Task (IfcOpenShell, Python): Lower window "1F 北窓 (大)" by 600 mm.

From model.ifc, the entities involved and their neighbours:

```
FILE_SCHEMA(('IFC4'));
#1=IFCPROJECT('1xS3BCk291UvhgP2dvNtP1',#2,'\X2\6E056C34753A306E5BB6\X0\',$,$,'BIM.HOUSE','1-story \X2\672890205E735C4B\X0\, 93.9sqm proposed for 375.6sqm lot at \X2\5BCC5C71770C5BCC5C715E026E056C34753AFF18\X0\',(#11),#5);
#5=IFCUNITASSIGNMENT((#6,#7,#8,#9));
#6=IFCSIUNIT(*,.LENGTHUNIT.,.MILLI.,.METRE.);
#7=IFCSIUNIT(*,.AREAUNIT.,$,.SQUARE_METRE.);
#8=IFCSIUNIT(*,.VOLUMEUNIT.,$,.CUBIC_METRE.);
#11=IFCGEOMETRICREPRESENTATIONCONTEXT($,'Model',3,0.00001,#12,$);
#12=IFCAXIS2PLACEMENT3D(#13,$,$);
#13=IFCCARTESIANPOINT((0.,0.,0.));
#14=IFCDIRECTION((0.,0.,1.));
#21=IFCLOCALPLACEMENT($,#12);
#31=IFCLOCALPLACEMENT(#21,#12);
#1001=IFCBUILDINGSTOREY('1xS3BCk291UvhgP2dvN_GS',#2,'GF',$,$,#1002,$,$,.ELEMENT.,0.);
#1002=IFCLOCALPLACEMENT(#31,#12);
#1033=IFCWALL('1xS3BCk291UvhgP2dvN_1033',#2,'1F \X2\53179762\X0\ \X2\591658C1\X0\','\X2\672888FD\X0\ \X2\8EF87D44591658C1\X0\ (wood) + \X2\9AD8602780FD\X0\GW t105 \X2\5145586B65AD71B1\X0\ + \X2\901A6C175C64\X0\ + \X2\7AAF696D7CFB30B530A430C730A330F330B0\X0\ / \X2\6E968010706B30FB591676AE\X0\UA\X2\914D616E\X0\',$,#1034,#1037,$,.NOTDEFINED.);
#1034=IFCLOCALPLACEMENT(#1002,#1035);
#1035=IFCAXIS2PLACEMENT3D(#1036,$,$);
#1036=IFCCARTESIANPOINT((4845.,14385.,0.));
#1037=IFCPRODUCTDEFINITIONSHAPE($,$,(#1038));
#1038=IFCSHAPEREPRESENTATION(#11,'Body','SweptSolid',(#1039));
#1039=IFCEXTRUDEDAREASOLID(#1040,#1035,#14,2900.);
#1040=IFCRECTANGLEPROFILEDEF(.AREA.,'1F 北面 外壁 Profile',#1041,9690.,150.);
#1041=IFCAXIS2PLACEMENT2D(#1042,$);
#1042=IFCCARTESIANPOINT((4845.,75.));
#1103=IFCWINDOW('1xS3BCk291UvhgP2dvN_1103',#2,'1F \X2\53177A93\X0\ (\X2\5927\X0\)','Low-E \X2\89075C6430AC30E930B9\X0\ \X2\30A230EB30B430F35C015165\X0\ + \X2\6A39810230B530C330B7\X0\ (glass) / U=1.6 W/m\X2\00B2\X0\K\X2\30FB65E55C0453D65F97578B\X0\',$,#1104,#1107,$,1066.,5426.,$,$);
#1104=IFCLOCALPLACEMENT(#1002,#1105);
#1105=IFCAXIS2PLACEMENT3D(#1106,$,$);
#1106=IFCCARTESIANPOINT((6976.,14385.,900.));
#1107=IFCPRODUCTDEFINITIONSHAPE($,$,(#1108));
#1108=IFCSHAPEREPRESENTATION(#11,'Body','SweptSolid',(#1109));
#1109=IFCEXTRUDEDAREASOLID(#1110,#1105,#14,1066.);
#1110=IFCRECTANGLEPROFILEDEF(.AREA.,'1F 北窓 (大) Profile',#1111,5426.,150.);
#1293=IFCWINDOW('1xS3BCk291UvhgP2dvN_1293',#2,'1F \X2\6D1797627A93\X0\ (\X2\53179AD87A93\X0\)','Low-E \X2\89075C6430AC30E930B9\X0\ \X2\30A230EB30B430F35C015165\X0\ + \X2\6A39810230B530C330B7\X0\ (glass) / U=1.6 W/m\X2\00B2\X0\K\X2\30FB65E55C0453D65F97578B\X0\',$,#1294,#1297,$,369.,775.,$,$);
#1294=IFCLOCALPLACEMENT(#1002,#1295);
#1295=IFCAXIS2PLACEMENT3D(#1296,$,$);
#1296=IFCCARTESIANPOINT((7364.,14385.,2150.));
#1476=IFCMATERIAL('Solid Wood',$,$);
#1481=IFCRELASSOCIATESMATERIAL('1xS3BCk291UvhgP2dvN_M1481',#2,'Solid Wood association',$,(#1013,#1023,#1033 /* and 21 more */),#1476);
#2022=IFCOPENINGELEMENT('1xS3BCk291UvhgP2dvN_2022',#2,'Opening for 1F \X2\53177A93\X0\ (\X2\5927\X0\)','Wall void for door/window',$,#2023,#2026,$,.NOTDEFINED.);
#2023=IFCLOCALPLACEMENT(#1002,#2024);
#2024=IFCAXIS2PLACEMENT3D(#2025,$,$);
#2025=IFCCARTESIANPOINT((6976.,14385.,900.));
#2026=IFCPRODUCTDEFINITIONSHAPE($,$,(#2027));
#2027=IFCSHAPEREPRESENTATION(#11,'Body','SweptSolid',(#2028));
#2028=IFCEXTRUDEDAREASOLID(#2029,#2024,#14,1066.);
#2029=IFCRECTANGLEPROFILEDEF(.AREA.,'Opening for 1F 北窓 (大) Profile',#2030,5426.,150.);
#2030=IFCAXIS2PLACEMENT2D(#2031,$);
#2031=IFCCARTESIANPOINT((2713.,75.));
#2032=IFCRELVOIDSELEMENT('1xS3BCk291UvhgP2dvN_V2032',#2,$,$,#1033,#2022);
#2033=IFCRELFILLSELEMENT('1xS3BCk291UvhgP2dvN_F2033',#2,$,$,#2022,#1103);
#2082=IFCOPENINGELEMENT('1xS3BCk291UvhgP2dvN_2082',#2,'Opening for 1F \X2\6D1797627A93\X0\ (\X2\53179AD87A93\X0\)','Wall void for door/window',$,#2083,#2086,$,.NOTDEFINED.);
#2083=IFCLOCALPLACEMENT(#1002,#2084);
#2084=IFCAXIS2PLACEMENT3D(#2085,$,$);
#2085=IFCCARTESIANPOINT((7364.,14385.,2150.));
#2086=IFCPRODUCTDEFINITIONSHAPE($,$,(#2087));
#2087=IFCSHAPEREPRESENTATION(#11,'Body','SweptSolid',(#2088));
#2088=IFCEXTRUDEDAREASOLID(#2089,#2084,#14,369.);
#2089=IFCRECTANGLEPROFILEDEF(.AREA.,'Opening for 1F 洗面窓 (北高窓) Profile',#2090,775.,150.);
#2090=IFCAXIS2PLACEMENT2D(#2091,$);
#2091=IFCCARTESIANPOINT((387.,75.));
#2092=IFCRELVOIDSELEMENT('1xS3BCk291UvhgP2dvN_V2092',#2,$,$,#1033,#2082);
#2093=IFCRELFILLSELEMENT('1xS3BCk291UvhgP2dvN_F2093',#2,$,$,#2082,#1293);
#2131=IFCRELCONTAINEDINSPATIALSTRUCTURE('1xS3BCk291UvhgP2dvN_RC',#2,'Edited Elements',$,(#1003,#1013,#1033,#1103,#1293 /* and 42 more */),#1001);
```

```python
import numpy as np
import ifcopenshell
import ifcopenshell.api.geometry
import ifcopenshell.util.placement
import ifcopenshell.util.unit

model = ifcopenshell.open("model.ifc")
unit_scale = ifcopenshell.util.unit.calculate_unit_scale(model)

window = model.by_guid("1xS3BCk291UvhgP2dvN_1103")
opening = window.FillsVoids[0].RelatingOpeningElement
dz = -600.0

shift = np.array([0.0, 0.0, dz])
# The window is not placed relative to its opening, so move both.
for product in (opening, window):
    matrix = ifcopenshell.util.placement.get_local_placement(product.ObjectPlacement)
    matrix[:3, 3] += shift
    ifcopenshell.api.geometry.edit_object_placement(model, product=product, matrix=matrix, is_si=False)

print(f"moved by {dz * unit_scale:+.3f} m")

model.write("model_rev.ifc")
```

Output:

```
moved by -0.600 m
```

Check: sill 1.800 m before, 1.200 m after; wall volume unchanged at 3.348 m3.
